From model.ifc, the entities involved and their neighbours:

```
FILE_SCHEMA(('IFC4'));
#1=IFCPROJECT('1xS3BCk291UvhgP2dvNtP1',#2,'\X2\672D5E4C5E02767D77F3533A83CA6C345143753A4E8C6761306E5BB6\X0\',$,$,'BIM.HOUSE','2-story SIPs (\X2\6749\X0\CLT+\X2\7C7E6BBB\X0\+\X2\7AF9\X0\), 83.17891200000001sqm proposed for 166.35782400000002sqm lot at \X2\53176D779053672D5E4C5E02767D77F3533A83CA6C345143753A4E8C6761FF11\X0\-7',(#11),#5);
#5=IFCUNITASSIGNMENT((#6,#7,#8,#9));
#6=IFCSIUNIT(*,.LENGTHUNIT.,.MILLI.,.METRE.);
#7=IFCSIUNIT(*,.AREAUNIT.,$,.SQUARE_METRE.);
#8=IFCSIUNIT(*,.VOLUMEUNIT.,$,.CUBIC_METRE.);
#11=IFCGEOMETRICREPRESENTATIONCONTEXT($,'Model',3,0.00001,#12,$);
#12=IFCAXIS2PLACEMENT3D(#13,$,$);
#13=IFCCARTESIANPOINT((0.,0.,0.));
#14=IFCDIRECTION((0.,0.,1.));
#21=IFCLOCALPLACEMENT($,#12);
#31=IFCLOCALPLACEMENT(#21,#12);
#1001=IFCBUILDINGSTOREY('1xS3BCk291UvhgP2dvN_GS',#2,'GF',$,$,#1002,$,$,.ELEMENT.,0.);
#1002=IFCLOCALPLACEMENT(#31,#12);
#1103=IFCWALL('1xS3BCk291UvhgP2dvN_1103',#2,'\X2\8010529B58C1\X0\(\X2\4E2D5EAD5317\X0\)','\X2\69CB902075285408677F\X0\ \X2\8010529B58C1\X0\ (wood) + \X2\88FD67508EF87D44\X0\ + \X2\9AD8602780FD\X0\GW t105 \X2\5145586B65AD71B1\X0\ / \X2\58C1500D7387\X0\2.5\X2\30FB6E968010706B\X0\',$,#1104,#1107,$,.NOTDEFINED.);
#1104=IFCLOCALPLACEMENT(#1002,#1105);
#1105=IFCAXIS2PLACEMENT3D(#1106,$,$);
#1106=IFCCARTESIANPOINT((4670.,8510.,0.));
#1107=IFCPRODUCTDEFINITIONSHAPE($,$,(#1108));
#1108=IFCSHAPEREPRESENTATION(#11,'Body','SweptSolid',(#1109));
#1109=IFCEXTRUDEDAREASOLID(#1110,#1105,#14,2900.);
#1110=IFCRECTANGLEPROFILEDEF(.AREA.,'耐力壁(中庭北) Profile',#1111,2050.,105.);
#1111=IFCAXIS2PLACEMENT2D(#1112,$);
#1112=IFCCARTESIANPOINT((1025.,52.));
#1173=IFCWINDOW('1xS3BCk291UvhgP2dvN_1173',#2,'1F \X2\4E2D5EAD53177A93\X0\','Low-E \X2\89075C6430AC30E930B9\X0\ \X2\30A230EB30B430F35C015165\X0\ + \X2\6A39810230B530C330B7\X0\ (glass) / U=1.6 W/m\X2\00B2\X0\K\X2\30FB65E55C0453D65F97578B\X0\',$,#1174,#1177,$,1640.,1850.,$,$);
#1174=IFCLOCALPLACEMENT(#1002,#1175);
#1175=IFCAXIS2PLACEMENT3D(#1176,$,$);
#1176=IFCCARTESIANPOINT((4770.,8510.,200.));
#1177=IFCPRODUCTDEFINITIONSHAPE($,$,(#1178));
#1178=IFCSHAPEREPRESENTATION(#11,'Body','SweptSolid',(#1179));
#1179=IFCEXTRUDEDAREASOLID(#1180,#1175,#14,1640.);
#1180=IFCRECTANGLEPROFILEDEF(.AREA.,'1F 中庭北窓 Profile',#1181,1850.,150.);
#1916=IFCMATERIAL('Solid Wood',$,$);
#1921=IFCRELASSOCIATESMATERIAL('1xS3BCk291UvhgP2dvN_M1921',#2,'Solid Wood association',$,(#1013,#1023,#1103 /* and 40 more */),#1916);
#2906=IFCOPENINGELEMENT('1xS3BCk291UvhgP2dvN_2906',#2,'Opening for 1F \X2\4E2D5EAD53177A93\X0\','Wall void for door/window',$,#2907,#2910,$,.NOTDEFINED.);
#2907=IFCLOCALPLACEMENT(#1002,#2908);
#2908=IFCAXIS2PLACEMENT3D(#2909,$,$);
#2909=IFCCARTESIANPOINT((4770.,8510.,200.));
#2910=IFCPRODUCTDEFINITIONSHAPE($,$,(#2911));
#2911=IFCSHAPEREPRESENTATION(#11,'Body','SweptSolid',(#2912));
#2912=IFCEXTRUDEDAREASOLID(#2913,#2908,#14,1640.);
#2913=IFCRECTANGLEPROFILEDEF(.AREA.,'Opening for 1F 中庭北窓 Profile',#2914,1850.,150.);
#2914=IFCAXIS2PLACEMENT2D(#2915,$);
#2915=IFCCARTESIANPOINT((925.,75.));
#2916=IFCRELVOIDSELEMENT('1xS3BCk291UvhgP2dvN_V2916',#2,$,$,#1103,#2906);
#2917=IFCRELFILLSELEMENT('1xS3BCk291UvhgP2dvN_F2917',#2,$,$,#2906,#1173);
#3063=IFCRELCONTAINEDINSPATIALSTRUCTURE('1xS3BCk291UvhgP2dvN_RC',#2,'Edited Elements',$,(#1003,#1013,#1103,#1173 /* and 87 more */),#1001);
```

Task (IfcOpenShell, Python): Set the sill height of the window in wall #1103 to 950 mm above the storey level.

```python
import numpy as np
import ifcopenshell
import ifcopenshell.api.geometry
import ifcopenshell.geom
import ifcopenshell.util.element
import ifcopenshell.util.placement
import ifcopenshell.util.shape
import ifcopenshell.util.unit

model = ifcopenshell.open("model.ifc")
unit_scale = ifcopenshell.util.unit.calculate_unit_scale(model)

window = model.by_guid("1xS3BCk291UvhgP2dvN_1173")
opening = window.FillsVoids[0].RelatingOpeningElement
storey = ifcopenshell.util.element.get_container(window, ifc_class="IfcBuildingStorey")
level = ifcopenshell.util.placement.get_local_placement(storey.ObjectPlacement)[2, 3]

# The opening's origin need not be at the sill, so measure its lowest point.
shape = ifcopenshell.geom.create_shape(ifcopenshell.geom.settings(), opening)
bottom = ifcopenshell.util.shape.get_shape_bottom_elevation(shape, shape.geometry) / unit_scale
dz = level + 950.0 - bottom

shift = np.array([0.0, 0.0, dz])
# The window is not placed relative to its opening, so move both.
for product in (opening, window):
    matrix = ifcopenshell.util.placement.get_local_placement(product.ObjectPlacement)
    matrix[:3, 3] += shift
    ifcopenshell.api.geometry.edit_object_placement(model, product=product, matrix=matrix, is_si=False)

print(f"moved by {dz * unit_scale:+.3f} m")

model.write("model_rev.ifc")
```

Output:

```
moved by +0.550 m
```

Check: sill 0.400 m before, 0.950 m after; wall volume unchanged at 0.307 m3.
